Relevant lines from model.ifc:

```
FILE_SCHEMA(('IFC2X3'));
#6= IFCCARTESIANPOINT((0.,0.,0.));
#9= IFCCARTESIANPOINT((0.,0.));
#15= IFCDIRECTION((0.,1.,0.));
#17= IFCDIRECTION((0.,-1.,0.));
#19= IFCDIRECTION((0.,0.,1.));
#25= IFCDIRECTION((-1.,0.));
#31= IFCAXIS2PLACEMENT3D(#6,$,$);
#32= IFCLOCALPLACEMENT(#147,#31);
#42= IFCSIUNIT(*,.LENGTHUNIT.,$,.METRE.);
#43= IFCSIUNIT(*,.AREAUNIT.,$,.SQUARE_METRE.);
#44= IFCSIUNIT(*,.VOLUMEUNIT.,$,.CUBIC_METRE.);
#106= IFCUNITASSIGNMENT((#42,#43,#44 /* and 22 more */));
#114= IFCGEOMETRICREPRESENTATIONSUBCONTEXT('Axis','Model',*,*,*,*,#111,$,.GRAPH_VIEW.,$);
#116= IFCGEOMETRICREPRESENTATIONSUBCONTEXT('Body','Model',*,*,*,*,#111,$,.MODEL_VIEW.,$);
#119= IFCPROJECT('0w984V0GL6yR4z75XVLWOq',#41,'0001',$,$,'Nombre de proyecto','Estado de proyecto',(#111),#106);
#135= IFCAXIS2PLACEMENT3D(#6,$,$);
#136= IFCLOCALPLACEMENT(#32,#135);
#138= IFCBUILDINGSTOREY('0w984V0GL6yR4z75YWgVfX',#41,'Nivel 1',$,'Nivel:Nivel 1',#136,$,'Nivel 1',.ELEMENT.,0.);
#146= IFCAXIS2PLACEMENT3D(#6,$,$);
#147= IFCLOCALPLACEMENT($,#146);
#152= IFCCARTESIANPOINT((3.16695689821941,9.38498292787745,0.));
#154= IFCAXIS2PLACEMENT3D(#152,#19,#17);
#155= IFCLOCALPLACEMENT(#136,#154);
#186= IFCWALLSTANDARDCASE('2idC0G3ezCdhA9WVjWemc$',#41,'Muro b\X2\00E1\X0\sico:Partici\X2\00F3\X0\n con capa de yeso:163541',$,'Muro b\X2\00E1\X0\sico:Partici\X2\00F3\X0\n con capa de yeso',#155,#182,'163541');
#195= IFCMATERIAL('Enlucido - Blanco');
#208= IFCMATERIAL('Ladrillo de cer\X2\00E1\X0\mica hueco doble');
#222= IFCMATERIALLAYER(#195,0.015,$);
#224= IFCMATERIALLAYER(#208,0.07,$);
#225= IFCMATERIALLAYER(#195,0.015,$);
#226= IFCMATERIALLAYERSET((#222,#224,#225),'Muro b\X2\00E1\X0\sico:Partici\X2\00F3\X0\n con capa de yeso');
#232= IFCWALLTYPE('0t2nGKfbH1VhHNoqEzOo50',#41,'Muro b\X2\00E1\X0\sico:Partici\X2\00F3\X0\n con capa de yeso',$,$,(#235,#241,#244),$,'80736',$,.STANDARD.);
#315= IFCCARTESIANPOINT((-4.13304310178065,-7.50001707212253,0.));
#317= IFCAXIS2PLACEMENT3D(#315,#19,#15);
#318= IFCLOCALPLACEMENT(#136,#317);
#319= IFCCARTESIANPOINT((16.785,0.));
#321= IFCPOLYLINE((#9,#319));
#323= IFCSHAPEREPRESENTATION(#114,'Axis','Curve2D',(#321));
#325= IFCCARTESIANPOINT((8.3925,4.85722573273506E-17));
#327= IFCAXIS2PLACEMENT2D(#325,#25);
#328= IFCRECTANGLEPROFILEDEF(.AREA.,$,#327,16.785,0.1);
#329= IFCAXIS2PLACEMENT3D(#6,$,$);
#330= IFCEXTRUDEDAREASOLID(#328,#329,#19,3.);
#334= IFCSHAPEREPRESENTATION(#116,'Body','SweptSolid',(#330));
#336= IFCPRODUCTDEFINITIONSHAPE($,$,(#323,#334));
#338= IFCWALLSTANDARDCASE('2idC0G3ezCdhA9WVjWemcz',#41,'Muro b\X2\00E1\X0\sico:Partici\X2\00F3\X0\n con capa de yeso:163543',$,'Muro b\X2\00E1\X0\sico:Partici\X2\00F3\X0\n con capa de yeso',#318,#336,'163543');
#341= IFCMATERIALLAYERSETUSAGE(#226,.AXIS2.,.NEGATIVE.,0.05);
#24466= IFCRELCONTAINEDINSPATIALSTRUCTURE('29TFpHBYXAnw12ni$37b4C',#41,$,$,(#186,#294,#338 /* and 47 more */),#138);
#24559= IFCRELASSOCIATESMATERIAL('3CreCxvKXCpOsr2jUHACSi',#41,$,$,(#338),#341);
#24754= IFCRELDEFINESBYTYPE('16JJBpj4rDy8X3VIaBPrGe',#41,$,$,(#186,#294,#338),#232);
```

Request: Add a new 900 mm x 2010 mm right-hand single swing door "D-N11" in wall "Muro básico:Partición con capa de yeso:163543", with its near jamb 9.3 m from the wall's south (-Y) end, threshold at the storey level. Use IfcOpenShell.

```python
import numpy as np
import ifcopenshell
import ifcopenshell.api.feature
import ifcopenshell.api.geometry
import ifcopenshell.api.root
import ifcopenshell.api.spatial
import ifcopenshell.api.type
import ifcopenshell.geom
import ifcopenshell.util.element
import ifcopenshell.util.placement
import ifcopenshell.util.representation
import ifcopenshell.util.shape
import ifcopenshell.util.unit

model = ifcopenshell.open("model.ifc")
unit_scale = ifcopenshell.util.unit.calculate_unit_scale(model)
settings = ifcopenshell.geom.settings()


def volume(element):
    """Net volume in cubic metres, openings subtracted."""
    shape = ifcopenshell.geom.create_shape(settings, element)
    return ifcopenshell.util.shape.get_volume(shape.geometry)


wall = model.by_guid("2idC0G3ezCdhA9WVjWemcz")
storey = ifcopenshell.util.element.get_container(wall, ifc_class="IfcBuildingStorey")
context = ifcopenshell.util.representation.get_context(model, "Model", "Body", "MODEL_VIEW")
before = volume(wall)

width, height, from_end, sill = 0.9, 2.01, 9.3, 0.0  # metres

# The wall runs along its own X axis, and the end named is its -X end.
wall_shape = ifcopenshell.geom.create_shape(settings, wall)
x, y, z = ifcopenshell.util.shape.get_vertices(wall_shape.geometry).T
start = x.min() + from_end
face, thickness = float(y.min()), float(y.max() - y.min())
wall_matrix = ifcopenshell.util.placement.get_local_placement(wall.ObjectPlacement)
level = ifcopenshell.util.placement.get_local_placement(storey.ObjectPlacement)[2, 3]


def in_wall(x, y):
    """Placement at x, y metres in the wall's axes, at sill height."""
    matrix = wall_matrix.copy()
    matrix[:, 3] = wall_matrix @ np.array([x / unit_scale, y / unit_scale, 0.0, 1.0])
    matrix[2, 3] = level + sill / unit_scale
    return matrix


# Opening: a box that overshoots both wall faces by 50 mm.
opening = ifcopenshell.api.root.create_entity(model, ifc_class="IfcOpeningElement")
box = ifcopenshell.api.geometry.add_wall_representation(
    model, context=context, length=width, height=height, thickness=thickness + 0.1
)
ifcopenshell.api.geometry.assign_representation(model, product=opening, representation=box)
ifcopenshell.api.geometry.edit_object_placement(model, product=opening, matrix=in_wall(start, face - 0.05), is_si=False)
ifcopenshell.api.feature.add_feature(model, feature=opening, element=wall)

door = ifcopenshell.api.root.create_entity(model, ifc_class="IfcDoor", name="D-N11")
door.OverallWidth, door.OverallHeight = width / unit_scale, height / unit_scale
body = ifcopenshell.api.geometry.add_door_representation(
    model,
    context=context,
    overall_width=door.OverallWidth,
    overall_height=door.OverallHeight,
    operation_type="SINGLE_SWING_RIGHT",
    lining_properties={"LiningDepth": thickness / unit_scale, "ThresholdDepth": thickness / unit_scale},
)
ifcopenshell.api.geometry.assign_representation(model, product=door, representation=body)
ifcopenshell.api.spatial.assign_container(model, products=[door], relating_structure=storey)
fills = ifcopenshell.api.feature.add_filling(model, opening=opening, element=door)
fills.OwnerHistory = door.OwnerHistory  # required in IFC2X3

# IFC2X3 keeps the operation on the door style.
style = ifcopenshell.api.root.create_entity(model, ifc_class="IfcDoorStyle", name="D-N11")
style.OperationType, style.ConstructionType = "SINGLE_SWING_RIGHT", "NOTDEFINED"
style.ParameterTakesPrecedence = style.Sizeable = False
ifcopenshell.api.type.assign_type(model, related_objects=[door], relating_type=style)

# The lining spans the wall, so the door starts at the wall face.
ifcopenshell.api.geometry.edit_object_placement(model, product=door, matrix=in_wall(start, face), is_si=False)

after = volume(wall)

print(f"wall volume {before:.3f} -> {after:.3f} m3")

model.write("model_updated.ifc")
```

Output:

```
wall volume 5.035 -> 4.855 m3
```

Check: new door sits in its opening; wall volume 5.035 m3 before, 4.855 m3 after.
